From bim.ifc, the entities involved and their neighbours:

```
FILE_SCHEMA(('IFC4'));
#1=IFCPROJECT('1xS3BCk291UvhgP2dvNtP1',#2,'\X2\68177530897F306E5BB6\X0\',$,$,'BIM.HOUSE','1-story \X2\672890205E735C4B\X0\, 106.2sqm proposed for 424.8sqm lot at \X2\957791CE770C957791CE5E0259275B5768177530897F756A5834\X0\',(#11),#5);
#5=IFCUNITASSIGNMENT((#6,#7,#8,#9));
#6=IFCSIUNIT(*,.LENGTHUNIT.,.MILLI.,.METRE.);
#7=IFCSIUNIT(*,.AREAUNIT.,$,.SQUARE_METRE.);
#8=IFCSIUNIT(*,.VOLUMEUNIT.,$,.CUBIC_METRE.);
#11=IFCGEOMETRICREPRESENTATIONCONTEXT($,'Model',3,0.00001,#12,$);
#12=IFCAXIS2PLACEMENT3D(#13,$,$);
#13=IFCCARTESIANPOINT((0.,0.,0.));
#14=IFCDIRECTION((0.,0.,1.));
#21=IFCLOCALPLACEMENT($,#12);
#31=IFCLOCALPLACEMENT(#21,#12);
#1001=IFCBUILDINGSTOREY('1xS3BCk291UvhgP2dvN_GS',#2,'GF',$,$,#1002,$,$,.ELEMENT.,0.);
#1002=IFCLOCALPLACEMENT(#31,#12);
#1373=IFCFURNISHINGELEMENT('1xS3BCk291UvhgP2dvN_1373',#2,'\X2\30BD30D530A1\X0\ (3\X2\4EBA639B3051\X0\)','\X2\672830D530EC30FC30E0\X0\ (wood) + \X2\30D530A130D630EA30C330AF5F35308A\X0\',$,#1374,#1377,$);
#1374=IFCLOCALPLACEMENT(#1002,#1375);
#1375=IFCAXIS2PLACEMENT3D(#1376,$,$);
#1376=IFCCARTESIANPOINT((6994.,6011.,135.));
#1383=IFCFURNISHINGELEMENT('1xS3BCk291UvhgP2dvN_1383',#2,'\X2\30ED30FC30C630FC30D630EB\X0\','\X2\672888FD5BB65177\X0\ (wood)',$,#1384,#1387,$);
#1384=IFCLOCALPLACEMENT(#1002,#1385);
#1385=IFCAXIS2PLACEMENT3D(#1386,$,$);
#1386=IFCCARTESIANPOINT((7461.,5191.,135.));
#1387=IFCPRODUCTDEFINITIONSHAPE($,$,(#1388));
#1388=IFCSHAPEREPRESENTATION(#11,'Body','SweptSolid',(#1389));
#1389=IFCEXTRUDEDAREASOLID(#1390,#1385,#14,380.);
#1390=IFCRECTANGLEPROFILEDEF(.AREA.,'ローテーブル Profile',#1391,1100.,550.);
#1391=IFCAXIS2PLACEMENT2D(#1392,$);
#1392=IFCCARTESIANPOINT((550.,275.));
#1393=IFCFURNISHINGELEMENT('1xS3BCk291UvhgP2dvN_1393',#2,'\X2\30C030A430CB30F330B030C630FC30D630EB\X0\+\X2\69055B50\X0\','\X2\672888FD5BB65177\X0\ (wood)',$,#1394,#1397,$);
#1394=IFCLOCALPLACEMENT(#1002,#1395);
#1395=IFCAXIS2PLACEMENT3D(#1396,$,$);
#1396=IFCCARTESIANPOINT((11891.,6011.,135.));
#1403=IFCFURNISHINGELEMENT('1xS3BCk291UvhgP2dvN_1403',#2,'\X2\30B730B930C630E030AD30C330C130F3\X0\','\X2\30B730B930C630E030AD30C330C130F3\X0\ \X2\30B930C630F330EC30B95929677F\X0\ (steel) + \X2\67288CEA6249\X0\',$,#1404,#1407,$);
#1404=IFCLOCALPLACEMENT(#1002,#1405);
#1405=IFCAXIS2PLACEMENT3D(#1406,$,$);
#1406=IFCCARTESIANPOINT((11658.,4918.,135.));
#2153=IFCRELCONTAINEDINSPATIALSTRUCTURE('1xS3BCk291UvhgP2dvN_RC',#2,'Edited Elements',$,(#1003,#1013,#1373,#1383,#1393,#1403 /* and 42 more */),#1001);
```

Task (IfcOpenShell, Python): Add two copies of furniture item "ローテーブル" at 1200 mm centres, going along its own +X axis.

```python
import ifcopenshell
import ifcopenshell.api.geometry
import ifcopenshell.api.root
import ifcopenshell.util.element
import ifcopenshell.util.placement
import ifcopenshell.util.unit

model = ifcopenshell.open("bim.ifc")
unit_scale = ifcopenshell.util.unit.calculate_unit_scale(model)


def reuse_history(source, copy):
    """copy_class also copies each property set's owner history, people and application; keep the originals."""
    for rel in copy.IsDefinedBy:
        if rel.is_a("IfcRelDefinesByProperties") and (history := rel.RelatingPropertyDefinition.OwnerHistory):
            rel.RelatingPropertyDefinition.OwnerHistory = source.OwnerHistory
            ifcopenshell.util.element.remove_deep2(model, history)


source = model.by_id(1383)
base = ifcopenshell.util.placement.get_local_placement(source.ObjectPlacement)
step = base[:3, 0] * 1.2 / unit_scale

for i in range(1, 3):
    copy = ifcopenshell.api.root.copy_class(model, product=source)
    copy.Representation = ifcopenshell.util.element.copy_deep(
        model, source.Representation, exclude=["IfcGeometricRepresentationContext", "IfcRepresentationMap"]
    )
    reuse_history(source, copy)
    matrix = base.copy()
    matrix[:3, 3] += i * step
    print("added at", matrix[:3, 3].round(3) + 0.0)
    ifcopenshell.api.geometry.edit_object_placement(model, product=copy, matrix=matrix, is_si=False)

model.write("bim-out.ifc")
```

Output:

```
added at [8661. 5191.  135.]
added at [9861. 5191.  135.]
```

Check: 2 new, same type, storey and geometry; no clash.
